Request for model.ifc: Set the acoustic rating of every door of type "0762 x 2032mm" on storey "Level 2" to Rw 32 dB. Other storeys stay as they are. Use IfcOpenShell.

First a look at what the model holds.

```python
import ifcopenshell
import ifcopenshell.util.element

model = ifcopenshell.open("model.ifc")
print(model.schema)
storey = next(s for s in model.by_type("IfcBuildingStorey") if s.Name == "Level 2")
doors = [e for e in ifcopenshell.util.element.get_decomposition(storey) if e.is_a("IfcDoor")]
seen = {}
for e in doors:
    element_type = ifcopenshell.util.element.get_type(e)
    key = (element_type.Name if element_type != e and element_type else None, ifcopenshell.util.element.get_pset(e, "Pset_DoorCommon", "AcousticRating"))
    seen[key] = seen.get(key, 0) + 1
for (name, value), count in sorted(seen.items(), key=str):
    print(count, "x", name, "|", value)
```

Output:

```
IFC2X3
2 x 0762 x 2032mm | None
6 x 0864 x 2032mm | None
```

```python
import ifcopenshell
import ifcopenshell.api.pset
import ifcopenshell.util.element

model = ifcopenshell.open("model.ifc")

storey = next(s for s in model.by_type("IfcBuildingStorey") if s.Name == "Level 2")
doors = [e for e in ifcopenshell.util.element.get_decomposition(storey) if e.is_a("IfcDoor")]

count = 0
for e in doors:
    element_type = ifcopenshell.util.element.get_type(e)
    if element_type in (None, e) or element_type.Name != "0762 x 2032mm":
        continue
    # add_pset returns the element's existing set when there is one.
    pset = ifcopenshell.api.pset.add_pset(model, product=e, name="Pset_DoorCommon")
    ifcopenshell.api.pset.edit_pset(model, pset=pset, properties={"AcousticRating": "Rw 32 dB"})
    count += 1

print(count, "doors updated")

model.write("model_edited.ifc")
```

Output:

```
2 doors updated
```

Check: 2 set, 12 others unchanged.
